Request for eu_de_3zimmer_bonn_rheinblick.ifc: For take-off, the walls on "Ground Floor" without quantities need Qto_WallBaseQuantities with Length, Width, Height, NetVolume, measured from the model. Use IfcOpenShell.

First a look at what the model holds.

```python
import ifcopenshell
import ifcopenshell.util.element
import ifcopenshell.util.unit

model = ifcopenshell.open("eu_de_3zimmer_bonn_rheinblick.ifc")
print(model.schema)
for unit_type in ("LENGTHUNIT", "AREAUNIT", "VOLUMEUNIT"):
    print(unit_type, ifcopenshell.util.unit.calculate_unit_scale(model, unit_type))
storey = next(s for s in model.by_type("IfcBuildingStorey") if s.Name == "Ground Floor")
walls = [e for e in ifcopenshell.util.element.get_decomposition(storey) if e.is_a("IfcWall")]
for e in sorted(walls, key=lambda e: e.id()):
    print(e.id(), e.is_a(), e.Name, list(ifcopenshell.util.element.get_psets(e, qtos_only=True)), sep=" | ")
```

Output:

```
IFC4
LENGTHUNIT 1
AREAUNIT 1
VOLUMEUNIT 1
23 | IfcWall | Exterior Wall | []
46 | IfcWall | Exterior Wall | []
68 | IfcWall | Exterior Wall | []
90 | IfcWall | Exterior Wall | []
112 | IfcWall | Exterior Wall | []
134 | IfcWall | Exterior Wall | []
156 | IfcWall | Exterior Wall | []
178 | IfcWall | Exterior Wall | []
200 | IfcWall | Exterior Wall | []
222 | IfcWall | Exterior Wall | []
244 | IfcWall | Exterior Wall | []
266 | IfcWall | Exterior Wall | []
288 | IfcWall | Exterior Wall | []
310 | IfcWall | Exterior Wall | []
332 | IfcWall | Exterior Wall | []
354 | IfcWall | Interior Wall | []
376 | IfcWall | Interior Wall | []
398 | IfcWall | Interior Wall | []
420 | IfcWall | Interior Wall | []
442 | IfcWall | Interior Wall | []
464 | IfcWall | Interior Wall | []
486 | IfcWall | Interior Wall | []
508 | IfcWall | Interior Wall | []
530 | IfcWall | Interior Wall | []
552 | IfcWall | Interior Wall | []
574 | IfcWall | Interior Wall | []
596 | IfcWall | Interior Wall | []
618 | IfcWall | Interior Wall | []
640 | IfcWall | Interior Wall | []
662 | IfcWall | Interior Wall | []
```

```python
import ifcopenshell
import ifcopenshell.api.pset
import ifcopenshell.geom
import ifcopenshell.util.element
import ifcopenshell.util.shape
import ifcopenshell.util.unit

model = ifcopenshell.open("eu_de_3zimmer_bonn_rheinblick.ifc")
unit_scale = ifcopenshell.util.unit.calculate_unit_scale(model)
volume_scale = ifcopenshell.util.unit.calculate_unit_scale(model, "VOLUMEUNIT")
settings = ifcopenshell.geom.settings()

storey = next(s for s in model.by_type("IfcBuildingStorey") if s.Name == "Ground Floor")
walls = [e for e in ifcopenshell.util.element.get_decomposition(storey) if e.is_a("IfcWall")]

for e in sorted(walls, key=lambda e: e.id()):
    if ifcopenshell.util.element.get_psets(e, qtos_only=True, should_inherit=False):
        continue
    # Geometry comes back in metres, in the element's own axes.
    shape = ifcopenshell.geom.create_shape(settings, e)
    values = {
        "Length": ifcopenshell.util.shape.get_x(shape.geometry) / unit_scale,
        "Width": ifcopenshell.util.shape.get_y(shape.geometry) / unit_scale,
        "Height": ifcopenshell.util.shape.get_z(shape.geometry) / unit_scale,
        "NetVolume": ifcopenshell.util.shape.get_volume(shape.geometry) / volume_scale,
    }
    qto = ifcopenshell.api.pset.add_qto(model, product=e, name="Qto_WallBaseQuantities")
    ifcopenshell.api.pset.edit_qto(model, qto=qto, properties=values)
    print(e.id(), {k: round(v, 3) for k, v in values.items()})

model.write("eu_de_3zimmer_bonn_rheinblick_rev.ifc")
```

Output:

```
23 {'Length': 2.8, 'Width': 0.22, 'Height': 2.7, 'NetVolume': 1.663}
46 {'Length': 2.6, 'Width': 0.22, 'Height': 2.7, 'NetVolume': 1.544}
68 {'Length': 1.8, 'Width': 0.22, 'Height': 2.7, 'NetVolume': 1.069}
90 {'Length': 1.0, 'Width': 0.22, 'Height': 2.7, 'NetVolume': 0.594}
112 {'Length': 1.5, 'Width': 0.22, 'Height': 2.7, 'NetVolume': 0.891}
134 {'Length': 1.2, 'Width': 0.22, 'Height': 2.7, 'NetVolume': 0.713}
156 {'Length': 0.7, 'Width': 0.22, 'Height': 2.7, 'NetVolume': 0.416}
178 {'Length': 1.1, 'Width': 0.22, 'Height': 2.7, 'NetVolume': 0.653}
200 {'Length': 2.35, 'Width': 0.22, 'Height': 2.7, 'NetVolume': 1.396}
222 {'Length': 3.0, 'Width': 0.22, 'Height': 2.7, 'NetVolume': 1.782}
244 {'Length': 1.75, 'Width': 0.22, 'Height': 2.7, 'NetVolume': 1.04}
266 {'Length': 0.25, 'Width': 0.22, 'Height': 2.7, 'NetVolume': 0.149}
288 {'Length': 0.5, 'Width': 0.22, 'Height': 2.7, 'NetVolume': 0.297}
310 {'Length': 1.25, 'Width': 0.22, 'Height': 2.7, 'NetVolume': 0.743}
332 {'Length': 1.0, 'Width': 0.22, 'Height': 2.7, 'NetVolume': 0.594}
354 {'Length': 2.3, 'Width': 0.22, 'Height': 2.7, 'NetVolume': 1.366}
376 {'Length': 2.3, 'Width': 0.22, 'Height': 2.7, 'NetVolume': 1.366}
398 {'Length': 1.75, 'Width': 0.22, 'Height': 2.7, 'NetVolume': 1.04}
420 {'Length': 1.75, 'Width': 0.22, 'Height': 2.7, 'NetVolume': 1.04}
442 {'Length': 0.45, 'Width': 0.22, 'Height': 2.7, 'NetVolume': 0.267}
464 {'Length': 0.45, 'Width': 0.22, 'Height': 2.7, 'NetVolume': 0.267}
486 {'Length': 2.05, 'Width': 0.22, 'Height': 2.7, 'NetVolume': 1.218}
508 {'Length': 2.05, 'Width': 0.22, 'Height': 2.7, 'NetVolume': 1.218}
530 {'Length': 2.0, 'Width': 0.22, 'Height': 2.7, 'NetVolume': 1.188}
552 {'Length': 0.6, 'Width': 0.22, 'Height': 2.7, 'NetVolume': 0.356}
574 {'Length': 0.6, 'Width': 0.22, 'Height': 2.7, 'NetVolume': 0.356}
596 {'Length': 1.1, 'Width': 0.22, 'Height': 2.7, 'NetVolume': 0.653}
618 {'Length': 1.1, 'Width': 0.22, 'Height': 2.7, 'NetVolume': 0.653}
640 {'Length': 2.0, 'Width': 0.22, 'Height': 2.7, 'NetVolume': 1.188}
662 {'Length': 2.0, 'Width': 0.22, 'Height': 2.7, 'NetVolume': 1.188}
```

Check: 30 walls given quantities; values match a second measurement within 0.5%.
